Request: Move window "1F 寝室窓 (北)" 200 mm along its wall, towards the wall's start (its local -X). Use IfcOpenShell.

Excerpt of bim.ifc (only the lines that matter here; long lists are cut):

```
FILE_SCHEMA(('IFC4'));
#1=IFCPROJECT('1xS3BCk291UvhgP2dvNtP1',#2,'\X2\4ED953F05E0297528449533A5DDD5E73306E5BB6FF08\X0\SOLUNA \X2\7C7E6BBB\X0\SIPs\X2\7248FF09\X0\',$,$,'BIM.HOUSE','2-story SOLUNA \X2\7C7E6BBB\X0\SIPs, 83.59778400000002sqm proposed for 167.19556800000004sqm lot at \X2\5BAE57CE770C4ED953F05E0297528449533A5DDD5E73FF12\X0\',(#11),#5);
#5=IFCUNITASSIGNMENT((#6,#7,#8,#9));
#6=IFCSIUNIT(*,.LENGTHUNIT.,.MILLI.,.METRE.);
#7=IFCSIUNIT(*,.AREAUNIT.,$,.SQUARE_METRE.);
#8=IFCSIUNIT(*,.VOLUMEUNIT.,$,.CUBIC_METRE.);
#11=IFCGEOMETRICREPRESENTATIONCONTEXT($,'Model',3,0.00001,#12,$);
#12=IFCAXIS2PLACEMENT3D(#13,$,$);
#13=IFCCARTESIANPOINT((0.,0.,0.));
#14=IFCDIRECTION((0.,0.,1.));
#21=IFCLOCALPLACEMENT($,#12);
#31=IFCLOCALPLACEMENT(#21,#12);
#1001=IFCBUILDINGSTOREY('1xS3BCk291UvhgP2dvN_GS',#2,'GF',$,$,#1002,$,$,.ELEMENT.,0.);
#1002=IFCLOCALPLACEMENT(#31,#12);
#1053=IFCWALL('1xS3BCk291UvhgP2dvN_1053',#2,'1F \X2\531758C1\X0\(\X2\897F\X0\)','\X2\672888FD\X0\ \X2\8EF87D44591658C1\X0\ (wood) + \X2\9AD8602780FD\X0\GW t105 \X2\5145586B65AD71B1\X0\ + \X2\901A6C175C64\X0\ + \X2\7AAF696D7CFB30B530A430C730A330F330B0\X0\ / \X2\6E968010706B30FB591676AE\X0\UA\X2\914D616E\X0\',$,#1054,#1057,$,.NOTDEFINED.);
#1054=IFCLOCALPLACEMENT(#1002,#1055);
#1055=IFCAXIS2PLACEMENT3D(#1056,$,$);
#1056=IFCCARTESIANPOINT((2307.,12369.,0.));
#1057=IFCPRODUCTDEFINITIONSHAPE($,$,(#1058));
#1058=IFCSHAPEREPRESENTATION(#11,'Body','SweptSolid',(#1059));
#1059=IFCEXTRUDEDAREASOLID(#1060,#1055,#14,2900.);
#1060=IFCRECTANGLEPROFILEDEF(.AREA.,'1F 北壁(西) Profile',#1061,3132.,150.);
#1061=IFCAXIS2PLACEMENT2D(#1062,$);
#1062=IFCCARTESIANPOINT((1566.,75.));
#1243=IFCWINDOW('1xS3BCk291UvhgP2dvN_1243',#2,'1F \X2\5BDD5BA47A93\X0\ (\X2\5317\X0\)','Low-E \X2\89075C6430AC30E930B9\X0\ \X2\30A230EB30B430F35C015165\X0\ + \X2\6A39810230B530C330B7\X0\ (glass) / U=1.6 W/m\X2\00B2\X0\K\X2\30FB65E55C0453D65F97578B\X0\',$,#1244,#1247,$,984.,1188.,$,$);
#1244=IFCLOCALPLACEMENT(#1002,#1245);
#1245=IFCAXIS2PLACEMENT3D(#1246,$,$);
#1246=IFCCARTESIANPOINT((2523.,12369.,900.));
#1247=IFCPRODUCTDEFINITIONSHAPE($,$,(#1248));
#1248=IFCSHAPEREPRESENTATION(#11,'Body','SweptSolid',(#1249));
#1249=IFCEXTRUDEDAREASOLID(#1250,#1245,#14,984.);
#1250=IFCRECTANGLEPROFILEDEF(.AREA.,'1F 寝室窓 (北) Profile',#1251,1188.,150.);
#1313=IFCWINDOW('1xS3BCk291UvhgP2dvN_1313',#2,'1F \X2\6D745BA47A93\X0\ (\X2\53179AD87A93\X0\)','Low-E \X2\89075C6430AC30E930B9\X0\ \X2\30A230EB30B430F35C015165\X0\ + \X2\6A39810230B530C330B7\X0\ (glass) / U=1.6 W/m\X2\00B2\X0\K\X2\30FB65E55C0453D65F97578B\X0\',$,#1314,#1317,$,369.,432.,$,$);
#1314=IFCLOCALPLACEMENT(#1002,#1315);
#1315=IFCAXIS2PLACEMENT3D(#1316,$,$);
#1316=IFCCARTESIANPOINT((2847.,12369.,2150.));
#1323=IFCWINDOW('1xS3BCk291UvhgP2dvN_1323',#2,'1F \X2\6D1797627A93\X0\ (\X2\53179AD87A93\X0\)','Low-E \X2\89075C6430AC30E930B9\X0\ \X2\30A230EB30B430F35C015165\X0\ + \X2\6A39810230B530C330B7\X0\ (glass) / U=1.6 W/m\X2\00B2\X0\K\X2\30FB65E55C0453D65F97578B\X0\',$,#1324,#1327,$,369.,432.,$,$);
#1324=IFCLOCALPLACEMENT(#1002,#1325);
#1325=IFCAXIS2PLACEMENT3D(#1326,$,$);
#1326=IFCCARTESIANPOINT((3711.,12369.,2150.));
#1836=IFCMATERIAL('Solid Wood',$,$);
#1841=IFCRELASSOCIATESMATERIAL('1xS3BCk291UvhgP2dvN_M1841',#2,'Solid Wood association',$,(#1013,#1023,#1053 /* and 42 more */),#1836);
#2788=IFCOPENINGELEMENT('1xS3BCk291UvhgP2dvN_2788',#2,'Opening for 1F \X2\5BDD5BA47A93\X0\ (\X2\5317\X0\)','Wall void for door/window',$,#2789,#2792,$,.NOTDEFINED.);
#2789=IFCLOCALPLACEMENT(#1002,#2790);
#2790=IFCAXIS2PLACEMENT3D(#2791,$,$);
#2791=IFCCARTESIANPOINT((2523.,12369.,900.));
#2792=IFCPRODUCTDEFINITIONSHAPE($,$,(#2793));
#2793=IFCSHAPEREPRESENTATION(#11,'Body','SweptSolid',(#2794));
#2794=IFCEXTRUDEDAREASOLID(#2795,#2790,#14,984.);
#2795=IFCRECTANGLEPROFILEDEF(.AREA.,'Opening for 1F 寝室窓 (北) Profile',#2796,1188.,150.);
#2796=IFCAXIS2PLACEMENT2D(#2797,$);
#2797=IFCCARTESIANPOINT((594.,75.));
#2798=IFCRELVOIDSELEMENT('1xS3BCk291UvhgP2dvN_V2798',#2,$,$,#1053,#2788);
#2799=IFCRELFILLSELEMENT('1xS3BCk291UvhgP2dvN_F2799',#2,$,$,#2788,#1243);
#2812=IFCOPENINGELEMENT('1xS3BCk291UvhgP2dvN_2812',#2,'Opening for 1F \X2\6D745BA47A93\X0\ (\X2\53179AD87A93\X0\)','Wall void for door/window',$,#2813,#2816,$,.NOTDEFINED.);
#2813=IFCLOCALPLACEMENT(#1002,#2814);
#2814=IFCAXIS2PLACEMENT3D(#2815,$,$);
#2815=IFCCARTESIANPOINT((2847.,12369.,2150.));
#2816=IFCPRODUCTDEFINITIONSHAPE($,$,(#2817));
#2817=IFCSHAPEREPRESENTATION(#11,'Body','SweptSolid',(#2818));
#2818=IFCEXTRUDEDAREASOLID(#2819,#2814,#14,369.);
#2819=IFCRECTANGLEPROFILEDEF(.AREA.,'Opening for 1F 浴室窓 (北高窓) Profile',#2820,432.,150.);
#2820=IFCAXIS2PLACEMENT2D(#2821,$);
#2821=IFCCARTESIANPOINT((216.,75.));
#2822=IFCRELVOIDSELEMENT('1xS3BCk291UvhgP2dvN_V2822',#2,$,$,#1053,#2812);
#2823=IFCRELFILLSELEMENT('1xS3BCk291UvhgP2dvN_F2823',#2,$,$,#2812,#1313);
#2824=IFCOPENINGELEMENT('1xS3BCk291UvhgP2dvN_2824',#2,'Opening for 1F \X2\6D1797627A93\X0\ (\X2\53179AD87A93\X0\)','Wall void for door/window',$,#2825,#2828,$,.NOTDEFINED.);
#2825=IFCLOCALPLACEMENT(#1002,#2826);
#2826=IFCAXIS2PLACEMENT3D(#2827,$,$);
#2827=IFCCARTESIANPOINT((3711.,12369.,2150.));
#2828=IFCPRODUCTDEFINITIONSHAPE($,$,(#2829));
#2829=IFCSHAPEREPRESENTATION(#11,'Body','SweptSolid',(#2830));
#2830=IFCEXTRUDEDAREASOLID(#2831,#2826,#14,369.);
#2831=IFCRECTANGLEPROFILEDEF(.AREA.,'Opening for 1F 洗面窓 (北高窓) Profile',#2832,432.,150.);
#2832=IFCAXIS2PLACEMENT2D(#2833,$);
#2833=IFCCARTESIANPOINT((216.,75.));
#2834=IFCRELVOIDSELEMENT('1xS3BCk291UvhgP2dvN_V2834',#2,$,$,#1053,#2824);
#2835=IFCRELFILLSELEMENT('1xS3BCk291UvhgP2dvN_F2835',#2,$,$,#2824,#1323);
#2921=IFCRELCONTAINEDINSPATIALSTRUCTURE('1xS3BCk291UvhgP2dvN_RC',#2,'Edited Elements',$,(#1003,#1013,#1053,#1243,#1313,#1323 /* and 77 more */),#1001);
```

```python
import ifcopenshell
import ifcopenshell.api.geometry
import ifcopenshell.util.placement
import ifcopenshell.util.unit

model = ifcopenshell.open("bim.ifc")
unit_scale = ifcopenshell.util.unit.calculate_unit_scale(model)

window = model.by_guid("1xS3BCk291UvhgP2dvN_1243")
opening = window.FillsVoids[0].RelatingOpeningElement
wall = opening.VoidsElements[0].RelatingBuildingElement

wall_matrix = ifcopenshell.util.placement.get_local_placement(wall.ObjectPlacement)
shift = wall_matrix[:3, 0] * -0.2 / unit_scale
before = ifcopenshell.util.placement.get_local_placement(window.ObjectPlacement)[:3, 3].copy()

# The window is not placed relative to its opening, so move both.
for product in (opening, window):
    matrix = ifcopenshell.util.placement.get_local_placement(product.ObjectPlacement)
    matrix[:3, 3] += shift
    ifcopenshell.api.geometry.edit_object_placement(model, product=product, matrix=matrix, is_si=False)

after = ifcopenshell.util.placement.get_local_placement(window.ObjectPlacement)[:3, 3]
print("window moved by", (after - before).round(3) + 0.0)

model.write("bim_updated.ifc")
```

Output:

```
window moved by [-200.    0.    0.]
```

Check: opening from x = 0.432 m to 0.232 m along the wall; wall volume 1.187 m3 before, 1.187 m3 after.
